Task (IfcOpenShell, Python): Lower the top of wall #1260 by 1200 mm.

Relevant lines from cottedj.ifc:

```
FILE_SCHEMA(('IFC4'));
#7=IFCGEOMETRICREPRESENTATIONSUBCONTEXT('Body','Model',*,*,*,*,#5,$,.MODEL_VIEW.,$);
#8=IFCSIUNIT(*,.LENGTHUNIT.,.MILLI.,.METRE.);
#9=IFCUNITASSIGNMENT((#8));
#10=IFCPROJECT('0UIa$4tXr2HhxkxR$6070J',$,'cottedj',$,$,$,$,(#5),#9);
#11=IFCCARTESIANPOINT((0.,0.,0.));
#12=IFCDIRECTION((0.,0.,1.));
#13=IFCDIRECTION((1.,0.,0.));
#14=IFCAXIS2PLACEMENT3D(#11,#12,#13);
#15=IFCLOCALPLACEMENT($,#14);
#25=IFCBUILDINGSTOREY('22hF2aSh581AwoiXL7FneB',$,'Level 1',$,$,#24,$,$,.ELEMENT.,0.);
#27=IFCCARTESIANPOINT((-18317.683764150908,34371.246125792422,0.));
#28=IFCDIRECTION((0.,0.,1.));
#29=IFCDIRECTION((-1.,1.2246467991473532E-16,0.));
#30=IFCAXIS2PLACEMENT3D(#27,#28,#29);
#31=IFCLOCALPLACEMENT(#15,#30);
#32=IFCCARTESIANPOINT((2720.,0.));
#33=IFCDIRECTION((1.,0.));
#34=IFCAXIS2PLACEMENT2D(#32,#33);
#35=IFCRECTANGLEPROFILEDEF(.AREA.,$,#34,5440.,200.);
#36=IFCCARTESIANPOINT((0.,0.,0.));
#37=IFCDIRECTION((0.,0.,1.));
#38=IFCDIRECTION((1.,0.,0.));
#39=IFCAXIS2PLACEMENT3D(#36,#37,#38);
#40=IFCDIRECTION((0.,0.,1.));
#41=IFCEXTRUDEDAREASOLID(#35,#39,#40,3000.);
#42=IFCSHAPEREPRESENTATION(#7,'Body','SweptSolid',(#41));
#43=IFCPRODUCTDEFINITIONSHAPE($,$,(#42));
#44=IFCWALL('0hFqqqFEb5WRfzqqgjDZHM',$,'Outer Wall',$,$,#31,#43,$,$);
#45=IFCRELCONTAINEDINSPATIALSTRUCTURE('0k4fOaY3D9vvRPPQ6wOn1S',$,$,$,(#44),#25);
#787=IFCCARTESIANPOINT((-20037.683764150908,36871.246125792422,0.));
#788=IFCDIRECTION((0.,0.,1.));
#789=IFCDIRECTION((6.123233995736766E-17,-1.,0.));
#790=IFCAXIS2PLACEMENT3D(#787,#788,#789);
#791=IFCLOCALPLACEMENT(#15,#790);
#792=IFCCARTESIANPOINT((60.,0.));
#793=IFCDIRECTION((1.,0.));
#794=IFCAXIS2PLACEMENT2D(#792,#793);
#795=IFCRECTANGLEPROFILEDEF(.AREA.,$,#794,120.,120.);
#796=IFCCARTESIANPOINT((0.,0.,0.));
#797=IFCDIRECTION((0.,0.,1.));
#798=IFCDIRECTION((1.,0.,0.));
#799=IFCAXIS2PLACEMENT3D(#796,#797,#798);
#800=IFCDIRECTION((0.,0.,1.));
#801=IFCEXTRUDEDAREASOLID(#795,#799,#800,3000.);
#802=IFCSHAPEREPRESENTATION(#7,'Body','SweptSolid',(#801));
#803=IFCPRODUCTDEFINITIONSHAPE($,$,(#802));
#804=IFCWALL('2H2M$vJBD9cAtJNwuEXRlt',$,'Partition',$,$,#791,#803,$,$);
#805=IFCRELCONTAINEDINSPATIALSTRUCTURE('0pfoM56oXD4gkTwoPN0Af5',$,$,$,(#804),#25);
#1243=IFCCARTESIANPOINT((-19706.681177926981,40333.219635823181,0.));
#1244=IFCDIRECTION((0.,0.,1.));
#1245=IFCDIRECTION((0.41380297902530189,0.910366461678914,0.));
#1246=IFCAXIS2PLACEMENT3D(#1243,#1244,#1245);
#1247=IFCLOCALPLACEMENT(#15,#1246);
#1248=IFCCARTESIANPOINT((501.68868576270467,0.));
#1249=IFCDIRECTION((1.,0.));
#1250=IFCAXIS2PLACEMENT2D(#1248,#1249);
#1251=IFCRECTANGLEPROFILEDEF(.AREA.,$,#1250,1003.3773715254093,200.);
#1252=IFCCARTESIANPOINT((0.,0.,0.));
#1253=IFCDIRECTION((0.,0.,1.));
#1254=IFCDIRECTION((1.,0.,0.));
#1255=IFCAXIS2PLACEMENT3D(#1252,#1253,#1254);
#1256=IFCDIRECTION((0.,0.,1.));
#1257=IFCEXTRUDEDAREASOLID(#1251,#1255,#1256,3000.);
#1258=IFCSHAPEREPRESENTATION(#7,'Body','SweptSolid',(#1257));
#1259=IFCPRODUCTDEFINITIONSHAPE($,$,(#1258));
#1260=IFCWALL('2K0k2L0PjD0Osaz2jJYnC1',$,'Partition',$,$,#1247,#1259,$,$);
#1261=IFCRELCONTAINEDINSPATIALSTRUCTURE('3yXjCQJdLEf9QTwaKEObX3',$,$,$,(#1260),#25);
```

```python
import ifcopenshell
import ifcopenshell.geom
import ifcopenshell.util.representation
import ifcopenshell.util.shape
import ifcopenshell.util.unit

model = ifcopenshell.open("cottedj.ifc")
unit_scale = ifcopenshell.util.unit.calculate_unit_scale(model)
settings = ifcopenshell.geom.settings()


def volume(element):
    """Net volume in cubic metres, openings subtracted."""
    shape = ifcopenshell.geom.create_shape(settings, element)
    return ifcopenshell.util.shape.get_volume(shape.geometry)


wall = model.by_guid("2K0k2L0PjD0Osaz2jJYnC1")
before = volume(wall)

body = ifcopenshell.util.representation.get_representation(wall, "Model", "Body")
solid = body.Items[0]
old_height = solid.Depth
solid.Depth -= 1.2 / unit_scale
after = volume(wall)

print(f"height {old_height:g} -> {solid.Depth:g}, volume {before:.3f} -> {after:.3f} m3")

model.write("cottedj_updated.ifc")
```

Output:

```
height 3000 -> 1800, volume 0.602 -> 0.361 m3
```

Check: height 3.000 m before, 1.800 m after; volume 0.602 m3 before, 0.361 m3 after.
